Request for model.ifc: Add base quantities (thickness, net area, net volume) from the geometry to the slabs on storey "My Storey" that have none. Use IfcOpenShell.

First a look at what the model holds.

```python
import ifcopenshell
import ifcopenshell.util.element
import ifcopenshell.util.unit

model = ifcopenshell.open("model.ifc")
print(model.schema)
for unit_type in ("LENGTHUNIT", "AREAUNIT", "VOLUMEUNIT"):
    print(unit_type, ifcopenshell.util.unit.calculate_unit_scale(model, unit_type))
storey = next(s for s in model.by_type("IfcBuildingStorey") if s.Name == "My Storey")
slabs = [e for e in ifcopenshell.util.element.get_decomposition(storey) if e.is_a("IfcSlab")]
for e in sorted(slabs, key=lambda e: e.id()):
    print(e.id(), e.is_a(), e.Name, list(ifcopenshell.util.element.get_psets(e, qtos_only=True)), sep=" | ")
```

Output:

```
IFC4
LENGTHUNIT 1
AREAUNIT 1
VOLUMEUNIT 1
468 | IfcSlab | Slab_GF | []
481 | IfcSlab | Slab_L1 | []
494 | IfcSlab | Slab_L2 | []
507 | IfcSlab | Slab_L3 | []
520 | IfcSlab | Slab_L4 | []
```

```python
import ifcopenshell
import ifcopenshell.api.pset
import ifcopenshell.geom
import ifcopenshell.util.element
import ifcopenshell.util.shape
import ifcopenshell.util.unit

model = ifcopenshell.open("model.ifc")
unit_scale = ifcopenshell.util.unit.calculate_unit_scale(model)
area_scale = ifcopenshell.util.unit.calculate_unit_scale(model, "AREAUNIT")
volume_scale = ifcopenshell.util.unit.calculate_unit_scale(model, "VOLUMEUNIT")
settings = ifcopenshell.geom.settings()

storey = next(s for s in model.by_type("IfcBuildingStorey") if s.Name == "My Storey")
slabs = [e for e in ifcopenshell.util.element.get_decomposition(storey) if e.is_a("IfcSlab")]

for e in sorted(slabs, key=lambda e: e.id()):
    if ifcopenshell.util.element.get_psets(e, qtos_only=True, should_inherit=False):
        continue
    # Geometry comes back in metres, in the element's own axes.
    shape = ifcopenshell.geom.create_shape(settings, e)
    values = {
        "Width": ifcopenshell.util.shape.get_z(shape.geometry) / unit_scale,
        "NetArea": ifcopenshell.util.shape.get_footprint_area(shape.geometry) / area_scale,
        "NetVolume": ifcopenshell.util.shape.get_volume(shape.geometry) / volume_scale,
    }
    qto = ifcopenshell.api.pset.add_qto(model, product=e, name="Qto_SlabBaseQuantities")
    ifcopenshell.api.pset.edit_qto(model, qto=qto, properties=values)
    print(e.id(), {k: round(v, 3) for k, v in values.items()})

model.write("model-out.ifc")
```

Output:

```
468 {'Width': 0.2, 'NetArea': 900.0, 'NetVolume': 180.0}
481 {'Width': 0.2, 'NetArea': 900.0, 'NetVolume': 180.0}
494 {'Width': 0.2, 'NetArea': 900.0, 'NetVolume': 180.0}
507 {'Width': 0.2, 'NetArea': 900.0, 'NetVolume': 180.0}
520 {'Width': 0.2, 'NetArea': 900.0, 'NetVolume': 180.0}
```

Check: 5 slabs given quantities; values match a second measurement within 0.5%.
